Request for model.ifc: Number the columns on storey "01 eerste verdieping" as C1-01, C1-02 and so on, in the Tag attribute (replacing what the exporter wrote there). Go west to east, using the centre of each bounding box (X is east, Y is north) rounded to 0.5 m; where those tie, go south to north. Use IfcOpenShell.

First a look at what the model holds.

```python
import ifcopenshell
import ifcopenshell.util.element
import ifcopenshell.util.placement

model = ifcopenshell.open("model.ifc")
print(model.schema)
storey = next(s for s in model.by_type("IfcBuildingStorey") if s.Name == "01 eerste verdieping")
columns = [e for e in ifcopenshell.util.element.get_decomposition(storey) if e.is_a("IfcColumn")]
for e in sorted(columns, key=lambda e: e.id()):
    origin = ifcopenshell.util.placement.get_local_placement(e.ObjectPlacement)[:3, 3]
    print(e.id(), e.Tag, e.Name, origin.round(2) + 0.0, sep=" | ")
```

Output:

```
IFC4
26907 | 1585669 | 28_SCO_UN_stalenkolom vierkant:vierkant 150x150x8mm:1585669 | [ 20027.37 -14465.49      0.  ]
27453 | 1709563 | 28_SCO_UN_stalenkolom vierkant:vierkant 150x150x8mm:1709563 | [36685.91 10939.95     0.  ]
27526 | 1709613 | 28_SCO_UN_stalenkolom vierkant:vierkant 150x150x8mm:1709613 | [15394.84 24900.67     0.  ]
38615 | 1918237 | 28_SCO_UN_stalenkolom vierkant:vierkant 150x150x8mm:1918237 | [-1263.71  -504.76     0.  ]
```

```python
import ifcopenshell
import ifcopenshell.geom
import ifcopenshell.util.element
import ifcopenshell.util.shape

model = ifcopenshell.open("model.ifc")
settings = ifcopenshell.geom.settings()
settings.set("use-world-coords", True)


def centre(element):
    shape = ifcopenshell.geom.create_shape(settings, element)
    return ifcopenshell.util.shape.get_bbox_centroid(shape.geometry)


storey = next(s for s in model.by_type("IfcBuildingStorey") if s.Name == "01 eerste verdieping")
columns = [e for e in ifcopenshell.util.element.get_decomposition(storey) if e.is_a("IfcColumn")]

# Insertion points can sit at a corner or the storey origin, so sort by the geometry (in metres).
centres = {e: centre(e) for e in columns}
columns.sort(key=lambda e: (round(centres[e][0] / 0.5), centres[e][1]))

for i, e in enumerate(columns, start=1):
    number = f"C1-{i:02d}"
    e.Tag = number
    print(e.id(), number)

model.write("model_rev.ifc")
```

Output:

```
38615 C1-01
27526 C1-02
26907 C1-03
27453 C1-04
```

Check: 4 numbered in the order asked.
